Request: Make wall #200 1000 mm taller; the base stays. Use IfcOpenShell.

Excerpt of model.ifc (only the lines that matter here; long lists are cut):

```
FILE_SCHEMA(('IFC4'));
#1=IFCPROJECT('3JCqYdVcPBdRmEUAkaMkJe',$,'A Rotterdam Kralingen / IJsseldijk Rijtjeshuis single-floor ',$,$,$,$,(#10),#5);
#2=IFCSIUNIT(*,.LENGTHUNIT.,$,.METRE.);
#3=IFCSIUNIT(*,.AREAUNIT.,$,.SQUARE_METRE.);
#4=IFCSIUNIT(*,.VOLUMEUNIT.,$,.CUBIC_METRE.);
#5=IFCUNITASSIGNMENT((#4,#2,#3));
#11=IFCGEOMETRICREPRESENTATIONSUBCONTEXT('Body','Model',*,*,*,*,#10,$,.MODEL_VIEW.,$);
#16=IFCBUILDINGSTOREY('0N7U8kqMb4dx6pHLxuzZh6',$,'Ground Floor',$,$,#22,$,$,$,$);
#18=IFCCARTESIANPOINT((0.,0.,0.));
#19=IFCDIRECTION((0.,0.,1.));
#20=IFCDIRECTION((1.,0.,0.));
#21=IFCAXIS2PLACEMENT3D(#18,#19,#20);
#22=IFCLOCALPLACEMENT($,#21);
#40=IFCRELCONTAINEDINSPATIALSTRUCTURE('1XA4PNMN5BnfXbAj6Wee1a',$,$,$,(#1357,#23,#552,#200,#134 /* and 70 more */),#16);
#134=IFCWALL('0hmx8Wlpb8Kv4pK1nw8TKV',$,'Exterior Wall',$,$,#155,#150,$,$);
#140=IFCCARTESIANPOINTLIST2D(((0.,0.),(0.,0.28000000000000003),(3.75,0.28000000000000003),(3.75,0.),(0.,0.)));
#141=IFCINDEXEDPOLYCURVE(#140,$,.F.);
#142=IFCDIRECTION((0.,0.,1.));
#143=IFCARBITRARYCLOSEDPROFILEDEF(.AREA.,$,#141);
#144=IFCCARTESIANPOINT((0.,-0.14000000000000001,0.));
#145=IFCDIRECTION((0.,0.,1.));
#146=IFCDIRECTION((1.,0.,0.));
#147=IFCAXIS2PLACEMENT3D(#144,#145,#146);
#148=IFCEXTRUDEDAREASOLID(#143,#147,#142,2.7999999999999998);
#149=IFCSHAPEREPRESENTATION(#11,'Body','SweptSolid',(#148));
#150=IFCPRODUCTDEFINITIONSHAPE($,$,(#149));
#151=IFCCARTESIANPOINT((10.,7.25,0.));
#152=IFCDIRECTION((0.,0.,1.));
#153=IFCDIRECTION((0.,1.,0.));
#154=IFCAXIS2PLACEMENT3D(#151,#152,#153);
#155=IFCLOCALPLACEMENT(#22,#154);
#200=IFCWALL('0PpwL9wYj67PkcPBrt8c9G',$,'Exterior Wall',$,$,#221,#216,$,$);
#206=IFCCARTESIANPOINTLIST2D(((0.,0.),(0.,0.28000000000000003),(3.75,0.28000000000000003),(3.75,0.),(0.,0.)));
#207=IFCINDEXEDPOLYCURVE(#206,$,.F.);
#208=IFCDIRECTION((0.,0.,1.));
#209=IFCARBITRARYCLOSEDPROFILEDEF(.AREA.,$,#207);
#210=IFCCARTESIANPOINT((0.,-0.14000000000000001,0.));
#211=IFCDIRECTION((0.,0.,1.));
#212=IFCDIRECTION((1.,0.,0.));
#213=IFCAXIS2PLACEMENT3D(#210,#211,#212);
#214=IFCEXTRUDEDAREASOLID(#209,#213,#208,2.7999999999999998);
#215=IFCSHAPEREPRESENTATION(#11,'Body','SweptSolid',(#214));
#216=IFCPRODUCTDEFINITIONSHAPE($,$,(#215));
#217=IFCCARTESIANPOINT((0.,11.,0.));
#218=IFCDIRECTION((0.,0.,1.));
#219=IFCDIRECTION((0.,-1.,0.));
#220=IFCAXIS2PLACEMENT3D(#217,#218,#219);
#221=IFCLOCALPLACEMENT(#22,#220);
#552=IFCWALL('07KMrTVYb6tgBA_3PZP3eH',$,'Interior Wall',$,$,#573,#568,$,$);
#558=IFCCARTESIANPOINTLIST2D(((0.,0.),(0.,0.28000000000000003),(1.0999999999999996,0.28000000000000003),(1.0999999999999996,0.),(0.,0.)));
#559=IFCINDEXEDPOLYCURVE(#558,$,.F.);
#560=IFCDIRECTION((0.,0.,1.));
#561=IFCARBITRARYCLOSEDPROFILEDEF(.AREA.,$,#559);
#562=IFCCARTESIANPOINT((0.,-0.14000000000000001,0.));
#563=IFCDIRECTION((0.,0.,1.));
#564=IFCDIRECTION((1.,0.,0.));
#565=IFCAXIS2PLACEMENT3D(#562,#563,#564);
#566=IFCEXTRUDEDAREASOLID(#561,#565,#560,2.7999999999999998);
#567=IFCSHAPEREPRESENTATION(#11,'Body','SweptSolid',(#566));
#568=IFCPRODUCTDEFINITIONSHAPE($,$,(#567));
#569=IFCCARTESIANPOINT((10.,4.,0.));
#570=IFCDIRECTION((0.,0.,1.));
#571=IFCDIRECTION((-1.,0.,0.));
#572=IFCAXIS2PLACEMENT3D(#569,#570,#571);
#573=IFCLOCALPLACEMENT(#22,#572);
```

```python
import ifcopenshell
import ifcopenshell.geom
import ifcopenshell.util.representation
import ifcopenshell.util.shape

model = ifcopenshell.open("model.ifc")
settings = ifcopenshell.geom.settings()


def volume(element):
    """Net volume in cubic metres, openings subtracted."""
    shape = ifcopenshell.geom.create_shape(settings, element)
    return ifcopenshell.util.shape.get_volume(shape.geometry)


wall = model.by_guid("0PpwL9wYj67PkcPBrt8c9G")
before = volume(wall)

body = ifcopenshell.util.representation.get_representation(wall, "Model", "Body")
solid = body.Items[0]
old_height = solid.Depth
solid.Depth += 1.0
after = volume(wall)

print(f"height {old_height:g} -> {solid.Depth:g}, volume {before:.3f} -> {after:.3f} m3")

model.write("model-out.ifc")
```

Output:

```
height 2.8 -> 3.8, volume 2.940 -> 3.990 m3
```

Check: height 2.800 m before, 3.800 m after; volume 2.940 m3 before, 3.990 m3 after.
